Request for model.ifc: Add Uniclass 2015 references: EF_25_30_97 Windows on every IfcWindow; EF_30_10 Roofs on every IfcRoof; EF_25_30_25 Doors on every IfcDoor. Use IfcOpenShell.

First a look at what the model holds.

```python
import ifcopenshell

model = ifcopenshell.open("model.ifc")
print(model.schema)
print("classifications:", [c.Name for c in model.by_type("IfcClassification")])
for ifc_class in ("IfcDoor", "IfcRoof", "IfcStair", "IfcWall", "IfcWindow"):
    print(ifc_class, len(model.by_type(ifc_class)))
```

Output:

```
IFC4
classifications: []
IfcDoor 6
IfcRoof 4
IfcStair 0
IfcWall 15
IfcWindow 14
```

```python
import ifcopenshell
import ifcopenshell.api.classification

model = ifcopenshell.open("model.ifc")

system = ifcopenshell.api.classification.add_classification(model, classification="Uniclass 2015")

codes = {
    "IfcWindow": ("EF_25_30_97", "Windows"),
    "IfcRoof": ("EF_30_10", "Roofs"),
    "IfcDoor": ("EF_25_30_25", "Doors"),
}
for ifc_class, (code, name) in codes.items():
    products = model.by_type(ifc_class)
    ifcopenshell.api.classification.add_reference(
        model, products=products, classification=system, identification=code, name=name
    )
    print(code, len(products))

model.write("model_edited.ifc")
```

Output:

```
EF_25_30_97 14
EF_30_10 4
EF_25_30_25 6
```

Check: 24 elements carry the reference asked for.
